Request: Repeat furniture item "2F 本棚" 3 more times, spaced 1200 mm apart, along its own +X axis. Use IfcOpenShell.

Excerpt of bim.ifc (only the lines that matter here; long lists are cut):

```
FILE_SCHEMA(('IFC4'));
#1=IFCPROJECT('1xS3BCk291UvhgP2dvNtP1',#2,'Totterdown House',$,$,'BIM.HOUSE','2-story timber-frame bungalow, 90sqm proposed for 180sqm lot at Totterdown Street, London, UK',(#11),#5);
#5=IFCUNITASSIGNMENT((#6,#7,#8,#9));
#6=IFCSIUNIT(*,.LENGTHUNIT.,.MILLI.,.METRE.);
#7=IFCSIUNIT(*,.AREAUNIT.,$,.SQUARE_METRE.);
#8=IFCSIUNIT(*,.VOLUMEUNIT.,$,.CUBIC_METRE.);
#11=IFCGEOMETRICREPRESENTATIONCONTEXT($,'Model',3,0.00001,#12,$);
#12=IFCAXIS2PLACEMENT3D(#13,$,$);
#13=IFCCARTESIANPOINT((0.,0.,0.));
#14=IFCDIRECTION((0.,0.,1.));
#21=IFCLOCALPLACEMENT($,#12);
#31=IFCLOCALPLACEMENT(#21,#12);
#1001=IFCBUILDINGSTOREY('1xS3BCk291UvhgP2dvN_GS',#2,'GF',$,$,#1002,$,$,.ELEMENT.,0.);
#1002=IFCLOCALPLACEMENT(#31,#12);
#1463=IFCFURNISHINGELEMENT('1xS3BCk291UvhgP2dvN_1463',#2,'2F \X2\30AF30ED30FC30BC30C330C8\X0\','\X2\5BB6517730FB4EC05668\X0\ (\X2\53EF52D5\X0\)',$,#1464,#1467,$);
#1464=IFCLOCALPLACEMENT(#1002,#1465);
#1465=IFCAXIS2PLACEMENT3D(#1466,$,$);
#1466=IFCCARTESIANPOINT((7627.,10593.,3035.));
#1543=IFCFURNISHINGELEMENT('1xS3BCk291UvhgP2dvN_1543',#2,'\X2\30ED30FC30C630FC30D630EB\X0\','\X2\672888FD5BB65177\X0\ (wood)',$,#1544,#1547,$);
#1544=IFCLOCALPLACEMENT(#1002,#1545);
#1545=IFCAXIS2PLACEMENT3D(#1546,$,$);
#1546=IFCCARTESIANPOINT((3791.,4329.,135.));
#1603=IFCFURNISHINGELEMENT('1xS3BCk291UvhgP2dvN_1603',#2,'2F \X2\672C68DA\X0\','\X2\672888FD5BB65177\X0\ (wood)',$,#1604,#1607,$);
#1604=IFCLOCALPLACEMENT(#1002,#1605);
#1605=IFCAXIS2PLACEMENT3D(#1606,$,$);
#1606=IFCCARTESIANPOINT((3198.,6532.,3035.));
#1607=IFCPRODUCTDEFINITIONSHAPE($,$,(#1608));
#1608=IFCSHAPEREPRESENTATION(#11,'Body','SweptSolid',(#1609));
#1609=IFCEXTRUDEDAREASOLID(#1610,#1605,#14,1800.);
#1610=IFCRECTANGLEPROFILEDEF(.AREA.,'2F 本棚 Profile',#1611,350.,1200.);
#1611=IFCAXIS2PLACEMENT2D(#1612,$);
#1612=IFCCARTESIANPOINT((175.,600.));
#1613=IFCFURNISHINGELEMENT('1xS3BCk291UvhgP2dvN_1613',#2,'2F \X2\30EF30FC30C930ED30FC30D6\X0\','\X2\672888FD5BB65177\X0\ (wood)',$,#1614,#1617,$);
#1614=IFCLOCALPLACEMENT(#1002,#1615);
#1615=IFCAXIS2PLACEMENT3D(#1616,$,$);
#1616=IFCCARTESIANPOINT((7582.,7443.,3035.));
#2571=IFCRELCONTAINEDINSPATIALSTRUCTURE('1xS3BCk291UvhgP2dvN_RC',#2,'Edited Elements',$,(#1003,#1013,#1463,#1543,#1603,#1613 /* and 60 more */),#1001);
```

```python
import ifcopenshell
import ifcopenshell.api.geometry
import ifcopenshell.api.root
import ifcopenshell.util.element
import ifcopenshell.util.placement
import ifcopenshell.util.unit

model = ifcopenshell.open("bim.ifc")
unit_scale = ifcopenshell.util.unit.calculate_unit_scale(model)


def reuse_history(source, copy):
    """copy_class also copies each property set's owner history, people and application; keep the originals."""
    for rel in copy.IsDefinedBy:
        if rel.is_a("IfcRelDefinesByProperties") and (history := rel.RelatingPropertyDefinition.OwnerHistory):
            rel.RelatingPropertyDefinition.OwnerHistory = source.OwnerHistory
            ifcopenshell.util.element.remove_deep2(model, history)


source = model.by_id(1603)
base = ifcopenshell.util.placement.get_local_placement(source.ObjectPlacement)
step = base[:3, 0] * 1.2 / unit_scale

for i in range(1, 4):
    copy = ifcopenshell.api.root.copy_class(model, product=source)
    copy.Representation = ifcopenshell.util.element.copy_deep(
        model, source.Representation, exclude=["IfcGeometricRepresentationContext", "IfcRepresentationMap"]
    )
    reuse_history(source, copy)
    matrix = base.copy()
    matrix[:3, 3] += i * step
    print("added at", matrix[:3, 3].round(3) + 0.0)
    ifcopenshell.api.geometry.edit_object_placement(model, product=copy, matrix=matrix, is_si=False)

model.write("bim_rev.ifc")
```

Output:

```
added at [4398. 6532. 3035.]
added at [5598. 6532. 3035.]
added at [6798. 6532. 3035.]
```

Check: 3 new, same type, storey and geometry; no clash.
